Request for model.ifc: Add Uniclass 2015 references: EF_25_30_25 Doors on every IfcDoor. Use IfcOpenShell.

First a look at what the model holds.

```python
import ifcopenshell

model = ifcopenshell.open("model.ifc")
print(model.schema)
print("classifications:", [c.Name for c in model.by_type("IfcClassification")])
for ifc_class in ("IfcDoor", "IfcRoof", "IfcStair", "IfcWall", "IfcWindow"):
    print(ifc_class, len(model.by_type(ifc_class)))
```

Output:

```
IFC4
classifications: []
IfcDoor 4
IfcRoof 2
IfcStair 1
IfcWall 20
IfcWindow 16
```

```python
import ifcopenshell
import ifcopenshell.api.classification

model = ifcopenshell.open("model.ifc")

system = ifcopenshell.api.classification.add_classification(model, classification="Uniclass 2015")

codes = {
    "IfcDoor": ("EF_25_30_25", "Doors"),
}
for ifc_class, (code, name) in codes.items():
    products = model.by_type(ifc_class)
    ifcopenshell.api.classification.add_reference(
        model, products=products, classification=system, identification=code, name=name
    )
    print(code, len(products))

model.write("model_rev.ifc")
```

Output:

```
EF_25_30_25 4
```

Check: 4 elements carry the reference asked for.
